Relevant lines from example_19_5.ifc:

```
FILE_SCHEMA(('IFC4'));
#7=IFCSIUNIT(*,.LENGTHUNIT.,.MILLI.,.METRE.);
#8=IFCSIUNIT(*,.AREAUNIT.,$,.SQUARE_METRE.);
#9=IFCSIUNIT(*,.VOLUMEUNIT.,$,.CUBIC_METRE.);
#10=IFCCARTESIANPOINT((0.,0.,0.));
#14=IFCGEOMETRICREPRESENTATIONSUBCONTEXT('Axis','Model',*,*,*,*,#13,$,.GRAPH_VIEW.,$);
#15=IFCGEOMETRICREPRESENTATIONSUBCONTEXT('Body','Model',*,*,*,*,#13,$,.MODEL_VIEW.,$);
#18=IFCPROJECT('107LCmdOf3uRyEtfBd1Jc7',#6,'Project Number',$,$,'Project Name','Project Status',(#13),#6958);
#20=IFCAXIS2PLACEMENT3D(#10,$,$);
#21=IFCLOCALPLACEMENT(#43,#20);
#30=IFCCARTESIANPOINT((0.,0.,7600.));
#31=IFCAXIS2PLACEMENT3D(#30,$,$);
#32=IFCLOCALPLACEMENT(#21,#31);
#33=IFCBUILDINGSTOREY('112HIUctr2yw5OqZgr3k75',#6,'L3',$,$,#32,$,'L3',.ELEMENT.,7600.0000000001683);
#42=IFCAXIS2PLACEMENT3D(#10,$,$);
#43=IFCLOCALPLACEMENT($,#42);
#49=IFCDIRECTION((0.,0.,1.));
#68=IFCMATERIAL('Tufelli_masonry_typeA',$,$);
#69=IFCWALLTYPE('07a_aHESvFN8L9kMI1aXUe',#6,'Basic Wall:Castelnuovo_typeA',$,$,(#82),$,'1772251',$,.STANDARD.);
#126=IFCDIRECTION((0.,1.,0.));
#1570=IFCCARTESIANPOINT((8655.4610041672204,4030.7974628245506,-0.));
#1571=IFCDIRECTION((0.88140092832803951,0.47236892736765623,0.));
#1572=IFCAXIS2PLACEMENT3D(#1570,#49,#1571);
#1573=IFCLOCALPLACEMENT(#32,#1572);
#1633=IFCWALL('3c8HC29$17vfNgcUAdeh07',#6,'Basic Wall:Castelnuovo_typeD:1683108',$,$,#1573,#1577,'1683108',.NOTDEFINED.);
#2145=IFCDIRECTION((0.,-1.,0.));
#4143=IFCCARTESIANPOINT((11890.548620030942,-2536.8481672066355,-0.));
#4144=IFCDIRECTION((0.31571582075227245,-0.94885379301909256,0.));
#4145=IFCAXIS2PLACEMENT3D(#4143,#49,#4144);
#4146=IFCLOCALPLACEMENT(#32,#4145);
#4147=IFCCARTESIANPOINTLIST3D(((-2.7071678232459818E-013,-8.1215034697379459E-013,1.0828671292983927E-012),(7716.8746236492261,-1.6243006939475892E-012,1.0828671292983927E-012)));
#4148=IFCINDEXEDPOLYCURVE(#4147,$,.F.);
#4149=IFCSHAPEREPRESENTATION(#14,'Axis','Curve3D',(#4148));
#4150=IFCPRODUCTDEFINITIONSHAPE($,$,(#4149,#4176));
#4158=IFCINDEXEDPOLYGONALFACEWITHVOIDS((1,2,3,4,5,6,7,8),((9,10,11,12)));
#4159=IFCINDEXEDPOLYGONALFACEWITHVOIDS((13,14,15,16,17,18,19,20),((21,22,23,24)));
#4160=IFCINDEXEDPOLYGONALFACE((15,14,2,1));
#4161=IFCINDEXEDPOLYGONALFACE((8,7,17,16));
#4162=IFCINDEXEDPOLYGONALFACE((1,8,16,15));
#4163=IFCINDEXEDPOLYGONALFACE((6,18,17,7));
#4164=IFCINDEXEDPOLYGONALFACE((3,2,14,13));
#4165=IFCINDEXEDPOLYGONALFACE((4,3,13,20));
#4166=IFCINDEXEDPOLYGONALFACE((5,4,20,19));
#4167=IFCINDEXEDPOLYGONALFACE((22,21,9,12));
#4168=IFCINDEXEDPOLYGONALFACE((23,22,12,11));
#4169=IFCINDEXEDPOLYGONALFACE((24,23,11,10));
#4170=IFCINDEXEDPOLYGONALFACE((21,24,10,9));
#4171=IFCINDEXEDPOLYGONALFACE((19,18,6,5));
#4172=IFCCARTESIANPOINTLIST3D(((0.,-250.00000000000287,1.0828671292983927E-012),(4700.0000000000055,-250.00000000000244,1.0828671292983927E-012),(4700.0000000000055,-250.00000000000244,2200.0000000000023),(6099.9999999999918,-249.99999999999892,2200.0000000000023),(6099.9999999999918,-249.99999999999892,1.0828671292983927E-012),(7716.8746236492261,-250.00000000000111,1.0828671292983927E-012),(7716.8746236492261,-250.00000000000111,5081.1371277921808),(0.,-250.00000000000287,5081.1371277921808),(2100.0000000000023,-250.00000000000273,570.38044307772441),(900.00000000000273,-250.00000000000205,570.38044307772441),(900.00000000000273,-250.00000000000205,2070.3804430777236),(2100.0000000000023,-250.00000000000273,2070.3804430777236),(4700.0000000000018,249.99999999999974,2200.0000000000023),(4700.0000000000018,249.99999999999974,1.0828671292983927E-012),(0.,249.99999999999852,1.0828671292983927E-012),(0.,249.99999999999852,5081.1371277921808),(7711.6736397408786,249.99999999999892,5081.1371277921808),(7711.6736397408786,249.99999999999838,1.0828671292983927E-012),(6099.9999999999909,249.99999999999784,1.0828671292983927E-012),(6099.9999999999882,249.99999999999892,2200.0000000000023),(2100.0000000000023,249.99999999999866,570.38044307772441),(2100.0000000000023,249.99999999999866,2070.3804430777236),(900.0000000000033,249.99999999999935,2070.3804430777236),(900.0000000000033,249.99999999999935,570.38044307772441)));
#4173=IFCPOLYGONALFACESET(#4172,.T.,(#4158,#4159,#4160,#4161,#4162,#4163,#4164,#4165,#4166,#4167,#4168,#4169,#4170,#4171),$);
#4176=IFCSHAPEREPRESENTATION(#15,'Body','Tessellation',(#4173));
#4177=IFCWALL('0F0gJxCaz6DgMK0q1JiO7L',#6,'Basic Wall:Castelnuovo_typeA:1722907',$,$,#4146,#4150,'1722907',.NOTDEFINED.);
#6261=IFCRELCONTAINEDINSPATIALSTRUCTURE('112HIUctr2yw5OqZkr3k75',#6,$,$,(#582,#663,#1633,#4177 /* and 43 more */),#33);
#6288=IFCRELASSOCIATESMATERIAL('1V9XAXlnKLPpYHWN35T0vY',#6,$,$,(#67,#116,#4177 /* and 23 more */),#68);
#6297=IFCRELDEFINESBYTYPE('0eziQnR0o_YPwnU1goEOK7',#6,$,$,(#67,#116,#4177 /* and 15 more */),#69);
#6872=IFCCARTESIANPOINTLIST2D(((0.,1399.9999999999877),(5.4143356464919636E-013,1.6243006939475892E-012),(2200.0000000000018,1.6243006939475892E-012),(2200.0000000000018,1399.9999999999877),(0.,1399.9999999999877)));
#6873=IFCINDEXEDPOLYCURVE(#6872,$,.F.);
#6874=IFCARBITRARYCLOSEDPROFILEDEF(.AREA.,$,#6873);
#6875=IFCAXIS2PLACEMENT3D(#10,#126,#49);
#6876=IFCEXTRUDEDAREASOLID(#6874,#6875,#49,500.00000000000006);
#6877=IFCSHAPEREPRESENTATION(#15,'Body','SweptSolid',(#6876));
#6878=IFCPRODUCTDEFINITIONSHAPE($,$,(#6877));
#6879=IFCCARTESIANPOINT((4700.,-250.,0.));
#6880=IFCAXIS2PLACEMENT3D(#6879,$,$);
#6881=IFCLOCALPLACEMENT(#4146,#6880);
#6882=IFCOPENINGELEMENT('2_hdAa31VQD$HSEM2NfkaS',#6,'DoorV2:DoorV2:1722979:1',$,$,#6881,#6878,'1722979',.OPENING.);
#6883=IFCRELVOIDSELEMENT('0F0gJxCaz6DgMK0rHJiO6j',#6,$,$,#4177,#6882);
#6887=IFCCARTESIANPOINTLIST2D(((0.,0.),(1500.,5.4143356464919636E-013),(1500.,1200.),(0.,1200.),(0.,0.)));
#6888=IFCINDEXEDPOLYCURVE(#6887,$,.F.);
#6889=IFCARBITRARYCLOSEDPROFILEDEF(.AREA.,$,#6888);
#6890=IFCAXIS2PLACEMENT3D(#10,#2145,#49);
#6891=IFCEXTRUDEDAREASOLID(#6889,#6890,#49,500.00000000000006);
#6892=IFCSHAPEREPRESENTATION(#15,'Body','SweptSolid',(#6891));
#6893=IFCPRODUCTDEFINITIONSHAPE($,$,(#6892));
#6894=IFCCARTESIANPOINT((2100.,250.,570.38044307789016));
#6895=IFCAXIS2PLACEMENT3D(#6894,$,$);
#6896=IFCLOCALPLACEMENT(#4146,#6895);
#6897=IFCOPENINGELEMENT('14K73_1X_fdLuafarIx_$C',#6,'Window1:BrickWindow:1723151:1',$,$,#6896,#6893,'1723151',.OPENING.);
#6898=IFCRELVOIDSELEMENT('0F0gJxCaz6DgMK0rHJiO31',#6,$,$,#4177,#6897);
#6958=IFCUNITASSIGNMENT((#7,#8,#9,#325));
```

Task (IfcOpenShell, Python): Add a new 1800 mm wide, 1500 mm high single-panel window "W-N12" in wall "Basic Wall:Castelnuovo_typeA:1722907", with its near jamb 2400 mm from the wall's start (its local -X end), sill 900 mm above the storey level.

```python
import numpy as np
import ifcopenshell
import ifcopenshell.api.feature
import ifcopenshell.api.geometry
import ifcopenshell.api.root
import ifcopenshell.api.spatial
import ifcopenshell.geom
import ifcopenshell.util.element
import ifcopenshell.util.placement
import ifcopenshell.util.representation
import ifcopenshell.util.shape
import ifcopenshell.util.unit

model = ifcopenshell.open("example_19_5.ifc")
unit_scale = ifcopenshell.util.unit.calculate_unit_scale(model)
settings = ifcopenshell.geom.settings()


def volume(element):
    """Net volume in cubic metres, openings subtracted."""
    shape = ifcopenshell.geom.create_shape(settings, element)
    return ifcopenshell.util.shape.get_volume(shape.geometry)


wall = model.by_id(4177)
storey = ifcopenshell.util.element.get_container(wall, ifc_class="IfcBuildingStorey")
context = ifcopenshell.util.representation.get_context(model, "Model", "Body", "MODEL_VIEW")
before = volume(wall)

width, height, from_end, sill = 1.8, 1.5, 2.4, 0.9  # metres

# The wall runs along its own X axis, and the end named is its -X end.
wall_shape = ifcopenshell.geom.create_shape(settings, wall)
x, y, z = ifcopenshell.util.shape.get_vertices(wall_shape.geometry).T
start = x.min() + from_end
face, thickness = float(y.min()), float(y.max() - y.min())
wall_matrix = ifcopenshell.util.placement.get_local_placement(wall.ObjectPlacement)
level = ifcopenshell.util.placement.get_local_placement(storey.ObjectPlacement)[2, 3]


def in_wall(x, y):
    """Placement at x, y metres in the wall's axes, at sill height."""
    matrix = wall_matrix.copy()
    matrix[:, 3] = wall_matrix @ np.array([x / unit_scale, y / unit_scale, 0.0, 1.0])
    matrix[2, 3] = level + sill / unit_scale
    return matrix


# Opening: a box that overshoots both wall faces by 50 mm.
opening = ifcopenshell.api.root.create_entity(model, ifc_class="IfcOpeningElement", predefined_type="OPENING")
box = ifcopenshell.api.geometry.add_wall_representation(
    model, context=context, length=width, height=height, thickness=thickness + 0.1
)
ifcopenshell.api.geometry.assign_representation(model, product=opening, representation=box)
ifcopenshell.api.geometry.edit_object_placement(model, product=opening, matrix=in_wall(start, face - 0.05), is_si=False)
ifcopenshell.api.feature.add_feature(model, feature=opening, element=wall)

window = ifcopenshell.api.root.create_entity(model, ifc_class="IfcWindow", name="W-N12", predefined_type="WINDOW")
window.OverallWidth, window.OverallHeight = width / unit_scale, height / unit_scale
window.PartitioningType = "SINGLE_PANEL"
body = ifcopenshell.api.geometry.add_window_representation(
    model,
    context=context,
    overall_width=window.OverallWidth,
    overall_height=window.OverallHeight,
    partition_type="SINGLE_PANEL",
)
ifcopenshell.api.geometry.assign_representation(model, product=window, representation=body)
ifcopenshell.api.spatial.assign_container(model, products=[window], relating_structure=storey)
ifcopenshell.api.feature.add_filling(model, opening=opening, element=window)

# Centre the window in the wall's thickness.
ifcopenshell.api.geometry.edit_object_placement(model, product=window, matrix=in_wall(start, face), is_si=False)
window_shape = ifcopenshell.geom.create_shape(settings, window)
depth = ifcopenshell.util.shape.get_vertices(window_shape.geometry)[:, 1]
offset = face + thickness / 2 - (depth.min() + depth.max()) / 2
ifcopenshell.api.geometry.edit_object_placement(model, product=window, matrix=in_wall(start, offset), is_si=False)

after = volume(wall)

print(f"wall volume {before:.3f} -> {after:.3f} m3")

model.write("example_19_5_edited.ifc")
```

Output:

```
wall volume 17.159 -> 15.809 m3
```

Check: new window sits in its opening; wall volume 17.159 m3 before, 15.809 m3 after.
